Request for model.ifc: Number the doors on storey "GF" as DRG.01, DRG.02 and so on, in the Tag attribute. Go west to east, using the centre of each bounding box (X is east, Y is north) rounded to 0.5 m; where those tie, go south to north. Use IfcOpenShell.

First a look at what the model holds.

```python
import ifcopenshell
import ifcopenshell.util.element
import ifcopenshell.util.placement

model = ifcopenshell.open("model.ifc")
print(model.schema)
storey = next(s for s in model.by_type("IfcBuildingStorey") if s.Name == "GF")
doors = [e for e in ifcopenshell.util.element.get_decomposition(storey) if e.is_a("IfcDoor")]
for e in sorted(doors, key=lambda e: e.id()):
    origin = ifcopenshell.util.placement.get_local_placement(e.ObjectPlacement)[:3, 3]
    print(e.id(), e.Tag, e.Name, origin.round(2) + 0.0, sep=" | ")
```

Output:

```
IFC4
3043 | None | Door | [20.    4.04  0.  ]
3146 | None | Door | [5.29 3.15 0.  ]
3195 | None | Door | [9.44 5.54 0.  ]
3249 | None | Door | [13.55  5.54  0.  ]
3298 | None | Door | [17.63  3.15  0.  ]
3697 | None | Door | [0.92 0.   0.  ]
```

```python
import ifcopenshell
import ifcopenshell.geom
import ifcopenshell.util.element
import ifcopenshell.util.shape

model = ifcopenshell.open("model.ifc")
settings = ifcopenshell.geom.settings()
settings.set("use-world-coords", True)


def centre(element):
    shape = ifcopenshell.geom.create_shape(settings, element)
    return ifcopenshell.util.shape.get_bbox_centroid(shape.geometry)


storey = next(s for s in model.by_type("IfcBuildingStorey") if s.Name == "GF")
doors = [e for e in ifcopenshell.util.element.get_decomposition(storey) if e.is_a("IfcDoor")]

# Insertion points can sit at a corner or the storey origin, so sort by the geometry (in metres).
centres = {e: centre(e) for e in doors}
doors.sort(key=lambda e: (round(centres[e][0] / 0.5), centres[e][1]))

for i, e in enumerate(doors, start=1):
    number = f"DRG.{i:02d}"
    e.Tag = number
    print(e.id(), number)

model.write("model_updated.ifc")
```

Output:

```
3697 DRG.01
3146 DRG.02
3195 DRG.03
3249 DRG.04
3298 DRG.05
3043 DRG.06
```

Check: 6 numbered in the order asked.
